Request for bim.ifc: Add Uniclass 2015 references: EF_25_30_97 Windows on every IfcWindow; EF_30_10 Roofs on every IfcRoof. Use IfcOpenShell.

First a look at what the model holds.

```python
import ifcopenshell

model = ifcopenshell.open("bim.ifc")
print(model.schema)
print("classifications:", [c.Name for c in model.by_type("IfcClassification")])
for ifc_class in ("IfcDoor", "IfcRoof", "IfcStair", "IfcWall", "IfcWindow"):
    print(ifc_class, len(model.by_type(ifc_class)))
```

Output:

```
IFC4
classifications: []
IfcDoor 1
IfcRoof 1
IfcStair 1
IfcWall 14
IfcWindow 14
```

```python
import ifcopenshell
import ifcopenshell.api.classification

model = ifcopenshell.open("bim.ifc")

system = ifcopenshell.api.classification.add_classification(model, classification="Uniclass 2015")

codes = {
    "IfcWindow": ("EF_25_30_97", "Windows"),
    "IfcRoof": ("EF_30_10", "Roofs"),
}
for ifc_class, (code, name) in codes.items():
    products = model.by_type(ifc_class)
    ifcopenshell.api.classification.add_reference(
        model, products=products, classification=system, identification=code, name=name
    )
    print(code, len(products))

model.write("bim-out.ifc")
```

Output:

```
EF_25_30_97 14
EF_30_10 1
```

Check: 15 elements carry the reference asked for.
